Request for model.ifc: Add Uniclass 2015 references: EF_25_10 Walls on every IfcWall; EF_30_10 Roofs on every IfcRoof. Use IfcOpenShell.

First a look at what the model holds.

```python
import ifcopenshell

model = ifcopenshell.open("model.ifc")
print(model.schema)
print("classifications:", [c.Name for c in model.by_type("IfcClassification")])
for ifc_class in ("IfcDoor", "IfcRoof", "IfcStair", "IfcWall", "IfcWindow"):
    print(ifc_class, len(model.by_type(ifc_class)))
```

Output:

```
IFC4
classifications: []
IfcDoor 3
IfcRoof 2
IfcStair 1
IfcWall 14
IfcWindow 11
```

```python
import ifcopenshell
import ifcopenshell.api.classification

model = ifcopenshell.open("model.ifc")

system = ifcopenshell.api.classification.add_classification(model, classification="Uniclass 2015")

codes = {
    "IfcWall": ("EF_25_10", "Walls"),
    "IfcRoof": ("EF_30_10", "Roofs"),
}
for ifc_class, (code, name) in codes.items():
    products = model.by_type(ifc_class)
    ifcopenshell.api.classification.add_reference(
        model, products=products, classification=system, identification=code, name=name
    )
    print(code, len(products))

model.write("model_updated.ifc")
```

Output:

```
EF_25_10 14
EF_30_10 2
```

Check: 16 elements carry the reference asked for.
